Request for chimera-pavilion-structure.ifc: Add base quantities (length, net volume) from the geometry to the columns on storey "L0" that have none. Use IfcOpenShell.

First a look at what the model holds.

```python
import ifcopenshell
import ifcopenshell.util.element
import ifcopenshell.util.unit

model = ifcopenshell.open("chimera-pavilion-structure.ifc")
print(model.schema)
for unit_type in ("LENGTHUNIT", "AREAUNIT", "VOLUMEUNIT"):
    print(unit_type, ifcopenshell.util.unit.calculate_unit_scale(model, unit_type))
storey = next(s for s in model.by_type("IfcBuildingStorey") if s.Name == "L0")
columns = [e for e in ifcopenshell.util.element.get_decomposition(storey) if e.is_a("IfcColumn")]
for e in sorted(columns, key=lambda e: e.id()):
    print(e.id(), e.is_a(), e.Name, list(ifcopenshell.util.element.get_psets(e, qtos_only=True)), sep=" | ")
```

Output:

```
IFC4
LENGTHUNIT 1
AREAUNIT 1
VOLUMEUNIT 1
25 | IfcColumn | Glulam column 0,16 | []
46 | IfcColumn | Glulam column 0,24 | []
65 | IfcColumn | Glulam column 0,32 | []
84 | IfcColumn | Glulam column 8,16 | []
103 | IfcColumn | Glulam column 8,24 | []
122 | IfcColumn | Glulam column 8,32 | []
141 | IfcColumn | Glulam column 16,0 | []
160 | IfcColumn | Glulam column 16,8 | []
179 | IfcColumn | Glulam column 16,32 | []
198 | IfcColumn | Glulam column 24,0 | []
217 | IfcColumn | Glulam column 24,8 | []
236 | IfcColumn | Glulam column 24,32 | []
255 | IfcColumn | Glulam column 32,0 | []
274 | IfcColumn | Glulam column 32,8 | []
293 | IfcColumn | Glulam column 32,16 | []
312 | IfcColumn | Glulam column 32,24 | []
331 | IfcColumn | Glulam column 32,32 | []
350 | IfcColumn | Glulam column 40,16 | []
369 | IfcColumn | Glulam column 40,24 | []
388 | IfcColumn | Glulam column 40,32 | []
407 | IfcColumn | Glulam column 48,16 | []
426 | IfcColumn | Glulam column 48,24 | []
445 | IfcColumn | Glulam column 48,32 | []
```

```python
import ifcopenshell
import ifcopenshell.api.pset
import ifcopenshell.geom
import ifcopenshell.util.element
import ifcopenshell.util.shape
import ifcopenshell.util.unit

model = ifcopenshell.open("chimera-pavilion-structure.ifc")
unit_scale = ifcopenshell.util.unit.calculate_unit_scale(model)
volume_scale = ifcopenshell.util.unit.calculate_unit_scale(model, "VOLUMEUNIT")
settings = ifcopenshell.geom.settings()

storey = next(s for s in model.by_type("IfcBuildingStorey") if s.Name == "L0")
columns = [e for e in ifcopenshell.util.element.get_decomposition(storey) if e.is_a("IfcColumn")]

for e in sorted(columns, key=lambda e: e.id()):
    if ifcopenshell.util.element.get_psets(e, qtos_only=True, should_inherit=False):
        continue
    # Geometry comes back in metres, in the element's own axes.
    shape = ifcopenshell.geom.create_shape(settings, e)
    values = {
        "Length": ifcopenshell.util.shape.get_z(shape.geometry) / unit_scale,
        "NetVolume": ifcopenshell.util.shape.get_volume(shape.geometry) / volume_scale,
    }
    qto = ifcopenshell.api.pset.add_qto(model, product=e, name="Qto_ColumnBaseQuantities")
    ifcopenshell.api.pset.edit_qto(model, qto=qto, properties=values)
    print(e.id(), {k: round(v, 3) for k, v in values.items()})

model.write("chimera-pavilion-structure_v2.ifc")
```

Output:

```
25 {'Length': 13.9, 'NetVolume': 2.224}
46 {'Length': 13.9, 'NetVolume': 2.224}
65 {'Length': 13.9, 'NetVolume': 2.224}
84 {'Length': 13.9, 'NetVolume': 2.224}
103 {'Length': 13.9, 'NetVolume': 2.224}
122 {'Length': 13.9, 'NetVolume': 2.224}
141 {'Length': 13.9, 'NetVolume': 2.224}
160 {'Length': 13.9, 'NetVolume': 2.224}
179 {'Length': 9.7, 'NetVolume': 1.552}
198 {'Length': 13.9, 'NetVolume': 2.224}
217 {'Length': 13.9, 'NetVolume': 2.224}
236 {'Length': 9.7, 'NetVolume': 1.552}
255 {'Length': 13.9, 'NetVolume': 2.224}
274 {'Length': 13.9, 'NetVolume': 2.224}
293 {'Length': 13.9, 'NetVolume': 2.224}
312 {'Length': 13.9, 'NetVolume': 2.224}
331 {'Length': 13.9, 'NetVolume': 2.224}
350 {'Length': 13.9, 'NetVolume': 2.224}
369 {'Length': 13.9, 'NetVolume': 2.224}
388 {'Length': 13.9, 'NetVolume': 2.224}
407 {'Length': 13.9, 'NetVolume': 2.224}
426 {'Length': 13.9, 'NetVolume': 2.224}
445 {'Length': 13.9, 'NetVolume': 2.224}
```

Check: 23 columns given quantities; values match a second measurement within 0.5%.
